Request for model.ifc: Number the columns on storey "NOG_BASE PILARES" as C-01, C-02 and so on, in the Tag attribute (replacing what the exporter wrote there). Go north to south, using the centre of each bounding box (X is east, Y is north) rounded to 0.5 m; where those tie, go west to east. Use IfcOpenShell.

First a look at what the model holds.

```python
import ifcopenshell
import ifcopenshell.util.element
import ifcopenshell.util.placement

model = ifcopenshell.open("model.ifc")
print(model.schema)
storey = next(s for s in model.by_type("IfcBuildingStorey") if s.Name == "NOG_BASE PILARES")
columns = [e for e in ifcopenshell.util.element.get_decomposition(storey) if e.is_a("IfcColumn")]
for e in sorted(columns, key=lambda e: e.id()):
    origin = ifcopenshell.util.placement.get_local_placement(e.ObjectPlacement)[:3, 3]
    print(e.id(), e.Tag, e.Name, origin.round(2) + 0.0, sep=" | ")
```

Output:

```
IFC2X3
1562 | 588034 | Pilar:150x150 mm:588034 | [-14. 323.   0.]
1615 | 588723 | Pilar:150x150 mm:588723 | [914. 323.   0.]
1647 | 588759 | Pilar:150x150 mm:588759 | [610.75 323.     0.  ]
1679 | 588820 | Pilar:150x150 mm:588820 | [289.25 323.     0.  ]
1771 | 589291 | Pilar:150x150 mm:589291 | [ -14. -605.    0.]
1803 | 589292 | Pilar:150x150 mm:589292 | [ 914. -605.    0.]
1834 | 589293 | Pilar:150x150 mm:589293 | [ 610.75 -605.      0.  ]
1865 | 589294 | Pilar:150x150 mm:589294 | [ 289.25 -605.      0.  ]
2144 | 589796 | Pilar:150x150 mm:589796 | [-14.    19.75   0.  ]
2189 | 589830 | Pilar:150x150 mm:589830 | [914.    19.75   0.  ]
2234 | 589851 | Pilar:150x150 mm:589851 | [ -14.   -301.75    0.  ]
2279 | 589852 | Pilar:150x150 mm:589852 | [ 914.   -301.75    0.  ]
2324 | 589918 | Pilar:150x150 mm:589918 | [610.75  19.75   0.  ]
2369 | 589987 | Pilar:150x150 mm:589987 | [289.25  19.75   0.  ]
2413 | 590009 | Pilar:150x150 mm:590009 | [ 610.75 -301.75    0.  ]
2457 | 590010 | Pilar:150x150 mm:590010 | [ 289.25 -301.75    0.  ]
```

```python
import ifcopenshell
import ifcopenshell.geom
import ifcopenshell.util.element
import ifcopenshell.util.shape

model = ifcopenshell.open("model.ifc")
settings = ifcopenshell.geom.settings()
settings.set("use-world-coords", True)


def centre(element):
    shape = ifcopenshell.geom.create_shape(settings, element)
    return ifcopenshell.util.shape.get_bbox_centroid(shape.geometry)


storey = next(s for s in model.by_type("IfcBuildingStorey") if s.Name == "NOG_BASE PILARES")
columns = [e for e in ifcopenshell.util.element.get_decomposition(storey) if e.is_a("IfcColumn")]

# Insertion points can sit at a corner or the storey origin, so sort by the geometry (in metres).
centres = {e: centre(e) for e in columns}
columns.sort(key=lambda e: (-round(centres[e][1] / 0.5), centres[e][0]))

for i, e in enumerate(columns, start=1):
    number = f"C-{i:02d}"
    e.Tag = number
    print(e.id(), number)

model.write("model-out.ifc")
```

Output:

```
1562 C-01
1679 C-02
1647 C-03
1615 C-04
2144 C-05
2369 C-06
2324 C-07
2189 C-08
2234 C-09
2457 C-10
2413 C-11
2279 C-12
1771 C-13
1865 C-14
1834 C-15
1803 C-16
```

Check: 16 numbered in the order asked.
